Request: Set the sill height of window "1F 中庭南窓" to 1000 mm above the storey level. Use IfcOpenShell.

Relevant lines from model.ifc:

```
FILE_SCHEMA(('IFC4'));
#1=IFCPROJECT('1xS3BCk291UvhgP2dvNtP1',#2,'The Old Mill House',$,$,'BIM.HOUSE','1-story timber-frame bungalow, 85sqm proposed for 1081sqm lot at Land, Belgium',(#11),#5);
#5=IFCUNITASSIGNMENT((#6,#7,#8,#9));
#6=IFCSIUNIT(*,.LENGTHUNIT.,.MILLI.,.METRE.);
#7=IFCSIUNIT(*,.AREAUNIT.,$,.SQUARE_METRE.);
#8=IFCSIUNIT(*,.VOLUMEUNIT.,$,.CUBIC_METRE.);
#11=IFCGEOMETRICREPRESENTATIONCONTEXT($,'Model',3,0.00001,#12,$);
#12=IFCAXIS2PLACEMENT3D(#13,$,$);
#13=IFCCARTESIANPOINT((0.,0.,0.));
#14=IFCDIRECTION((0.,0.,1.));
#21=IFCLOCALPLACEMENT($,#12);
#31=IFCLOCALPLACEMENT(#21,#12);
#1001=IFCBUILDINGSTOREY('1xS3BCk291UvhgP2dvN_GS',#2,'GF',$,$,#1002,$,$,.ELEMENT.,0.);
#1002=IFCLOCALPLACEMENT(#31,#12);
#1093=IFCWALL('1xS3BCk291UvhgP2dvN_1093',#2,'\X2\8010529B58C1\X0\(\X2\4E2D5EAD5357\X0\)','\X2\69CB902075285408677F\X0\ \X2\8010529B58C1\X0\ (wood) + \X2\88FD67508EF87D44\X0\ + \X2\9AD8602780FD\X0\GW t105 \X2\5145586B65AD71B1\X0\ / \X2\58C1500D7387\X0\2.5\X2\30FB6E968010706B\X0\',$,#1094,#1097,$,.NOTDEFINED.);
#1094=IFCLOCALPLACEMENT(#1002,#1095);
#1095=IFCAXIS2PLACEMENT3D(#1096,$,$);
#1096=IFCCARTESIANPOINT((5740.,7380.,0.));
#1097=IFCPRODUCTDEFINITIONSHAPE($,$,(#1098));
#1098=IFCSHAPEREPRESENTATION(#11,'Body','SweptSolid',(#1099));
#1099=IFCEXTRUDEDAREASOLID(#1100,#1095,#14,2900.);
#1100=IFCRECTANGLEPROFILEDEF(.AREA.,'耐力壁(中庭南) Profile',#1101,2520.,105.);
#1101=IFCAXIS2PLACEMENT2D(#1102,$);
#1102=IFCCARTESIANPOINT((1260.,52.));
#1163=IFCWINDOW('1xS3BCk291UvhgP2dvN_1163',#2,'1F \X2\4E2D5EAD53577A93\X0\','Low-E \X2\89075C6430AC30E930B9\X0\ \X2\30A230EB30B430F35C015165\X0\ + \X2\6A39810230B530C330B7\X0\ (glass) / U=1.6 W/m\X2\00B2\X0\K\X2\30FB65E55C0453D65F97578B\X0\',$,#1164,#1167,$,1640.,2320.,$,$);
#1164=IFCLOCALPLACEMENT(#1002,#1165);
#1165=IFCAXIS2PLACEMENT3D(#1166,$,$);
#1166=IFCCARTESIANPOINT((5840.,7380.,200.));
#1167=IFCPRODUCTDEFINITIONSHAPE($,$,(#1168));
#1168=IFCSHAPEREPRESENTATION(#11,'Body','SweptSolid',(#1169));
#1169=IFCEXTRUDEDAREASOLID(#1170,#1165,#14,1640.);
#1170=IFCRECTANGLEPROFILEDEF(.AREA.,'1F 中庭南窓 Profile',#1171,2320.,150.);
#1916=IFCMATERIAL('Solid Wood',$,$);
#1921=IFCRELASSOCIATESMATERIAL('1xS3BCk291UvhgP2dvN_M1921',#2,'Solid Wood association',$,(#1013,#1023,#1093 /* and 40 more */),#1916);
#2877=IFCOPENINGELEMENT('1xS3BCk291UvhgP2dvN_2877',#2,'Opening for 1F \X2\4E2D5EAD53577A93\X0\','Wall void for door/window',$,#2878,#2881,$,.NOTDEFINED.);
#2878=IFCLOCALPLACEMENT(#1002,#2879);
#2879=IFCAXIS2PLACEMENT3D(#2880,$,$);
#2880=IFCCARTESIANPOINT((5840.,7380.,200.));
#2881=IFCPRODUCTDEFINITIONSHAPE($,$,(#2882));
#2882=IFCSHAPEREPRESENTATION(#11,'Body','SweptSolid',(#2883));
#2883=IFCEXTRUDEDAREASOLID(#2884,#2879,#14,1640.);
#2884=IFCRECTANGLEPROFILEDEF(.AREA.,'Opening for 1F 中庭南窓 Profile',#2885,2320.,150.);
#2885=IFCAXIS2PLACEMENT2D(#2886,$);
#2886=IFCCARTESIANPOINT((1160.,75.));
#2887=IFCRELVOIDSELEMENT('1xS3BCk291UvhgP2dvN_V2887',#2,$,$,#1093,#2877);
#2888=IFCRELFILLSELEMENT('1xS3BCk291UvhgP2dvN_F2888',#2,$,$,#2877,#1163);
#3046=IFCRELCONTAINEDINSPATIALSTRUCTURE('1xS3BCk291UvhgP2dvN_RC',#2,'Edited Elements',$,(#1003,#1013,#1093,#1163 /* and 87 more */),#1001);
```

```python
import numpy as np
import ifcopenshell
import ifcopenshell.api.geometry
import ifcopenshell.geom
import ifcopenshell.util.element
import ifcopenshell.util.placement
import ifcopenshell.util.shape
import ifcopenshell.util.unit

model = ifcopenshell.open("model.ifc")
unit_scale = ifcopenshell.util.unit.calculate_unit_scale(model)

window = model.by_guid("1xS3BCk291UvhgP2dvN_1163")
opening = window.FillsVoids[0].RelatingOpeningElement
storey = ifcopenshell.util.element.get_container(window, ifc_class="IfcBuildingStorey")
level = ifcopenshell.util.placement.get_local_placement(storey.ObjectPlacement)[2, 3]

# The opening's origin need not be at the sill, so measure its lowest point.
shape = ifcopenshell.geom.create_shape(ifcopenshell.geom.settings(), opening)
bottom = ifcopenshell.util.shape.get_shape_bottom_elevation(shape, shape.geometry) / unit_scale
dz = level + 1000.0 - bottom

shift = np.array([0.0, 0.0, dz])
# The window is not placed relative to its opening, so move both.
for product in (opening, window):
    matrix = ifcopenshell.util.placement.get_local_placement(product.ObjectPlacement)
    matrix[:3, 3] += shift
    ifcopenshell.api.geometry.edit_object_placement(model, product=product, matrix=matrix, is_si=False)

print(f"moved by {dz * unit_scale:+.3f} m")

model.write("model_v2.ifc")
```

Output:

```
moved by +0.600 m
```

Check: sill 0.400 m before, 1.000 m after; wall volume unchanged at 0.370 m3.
